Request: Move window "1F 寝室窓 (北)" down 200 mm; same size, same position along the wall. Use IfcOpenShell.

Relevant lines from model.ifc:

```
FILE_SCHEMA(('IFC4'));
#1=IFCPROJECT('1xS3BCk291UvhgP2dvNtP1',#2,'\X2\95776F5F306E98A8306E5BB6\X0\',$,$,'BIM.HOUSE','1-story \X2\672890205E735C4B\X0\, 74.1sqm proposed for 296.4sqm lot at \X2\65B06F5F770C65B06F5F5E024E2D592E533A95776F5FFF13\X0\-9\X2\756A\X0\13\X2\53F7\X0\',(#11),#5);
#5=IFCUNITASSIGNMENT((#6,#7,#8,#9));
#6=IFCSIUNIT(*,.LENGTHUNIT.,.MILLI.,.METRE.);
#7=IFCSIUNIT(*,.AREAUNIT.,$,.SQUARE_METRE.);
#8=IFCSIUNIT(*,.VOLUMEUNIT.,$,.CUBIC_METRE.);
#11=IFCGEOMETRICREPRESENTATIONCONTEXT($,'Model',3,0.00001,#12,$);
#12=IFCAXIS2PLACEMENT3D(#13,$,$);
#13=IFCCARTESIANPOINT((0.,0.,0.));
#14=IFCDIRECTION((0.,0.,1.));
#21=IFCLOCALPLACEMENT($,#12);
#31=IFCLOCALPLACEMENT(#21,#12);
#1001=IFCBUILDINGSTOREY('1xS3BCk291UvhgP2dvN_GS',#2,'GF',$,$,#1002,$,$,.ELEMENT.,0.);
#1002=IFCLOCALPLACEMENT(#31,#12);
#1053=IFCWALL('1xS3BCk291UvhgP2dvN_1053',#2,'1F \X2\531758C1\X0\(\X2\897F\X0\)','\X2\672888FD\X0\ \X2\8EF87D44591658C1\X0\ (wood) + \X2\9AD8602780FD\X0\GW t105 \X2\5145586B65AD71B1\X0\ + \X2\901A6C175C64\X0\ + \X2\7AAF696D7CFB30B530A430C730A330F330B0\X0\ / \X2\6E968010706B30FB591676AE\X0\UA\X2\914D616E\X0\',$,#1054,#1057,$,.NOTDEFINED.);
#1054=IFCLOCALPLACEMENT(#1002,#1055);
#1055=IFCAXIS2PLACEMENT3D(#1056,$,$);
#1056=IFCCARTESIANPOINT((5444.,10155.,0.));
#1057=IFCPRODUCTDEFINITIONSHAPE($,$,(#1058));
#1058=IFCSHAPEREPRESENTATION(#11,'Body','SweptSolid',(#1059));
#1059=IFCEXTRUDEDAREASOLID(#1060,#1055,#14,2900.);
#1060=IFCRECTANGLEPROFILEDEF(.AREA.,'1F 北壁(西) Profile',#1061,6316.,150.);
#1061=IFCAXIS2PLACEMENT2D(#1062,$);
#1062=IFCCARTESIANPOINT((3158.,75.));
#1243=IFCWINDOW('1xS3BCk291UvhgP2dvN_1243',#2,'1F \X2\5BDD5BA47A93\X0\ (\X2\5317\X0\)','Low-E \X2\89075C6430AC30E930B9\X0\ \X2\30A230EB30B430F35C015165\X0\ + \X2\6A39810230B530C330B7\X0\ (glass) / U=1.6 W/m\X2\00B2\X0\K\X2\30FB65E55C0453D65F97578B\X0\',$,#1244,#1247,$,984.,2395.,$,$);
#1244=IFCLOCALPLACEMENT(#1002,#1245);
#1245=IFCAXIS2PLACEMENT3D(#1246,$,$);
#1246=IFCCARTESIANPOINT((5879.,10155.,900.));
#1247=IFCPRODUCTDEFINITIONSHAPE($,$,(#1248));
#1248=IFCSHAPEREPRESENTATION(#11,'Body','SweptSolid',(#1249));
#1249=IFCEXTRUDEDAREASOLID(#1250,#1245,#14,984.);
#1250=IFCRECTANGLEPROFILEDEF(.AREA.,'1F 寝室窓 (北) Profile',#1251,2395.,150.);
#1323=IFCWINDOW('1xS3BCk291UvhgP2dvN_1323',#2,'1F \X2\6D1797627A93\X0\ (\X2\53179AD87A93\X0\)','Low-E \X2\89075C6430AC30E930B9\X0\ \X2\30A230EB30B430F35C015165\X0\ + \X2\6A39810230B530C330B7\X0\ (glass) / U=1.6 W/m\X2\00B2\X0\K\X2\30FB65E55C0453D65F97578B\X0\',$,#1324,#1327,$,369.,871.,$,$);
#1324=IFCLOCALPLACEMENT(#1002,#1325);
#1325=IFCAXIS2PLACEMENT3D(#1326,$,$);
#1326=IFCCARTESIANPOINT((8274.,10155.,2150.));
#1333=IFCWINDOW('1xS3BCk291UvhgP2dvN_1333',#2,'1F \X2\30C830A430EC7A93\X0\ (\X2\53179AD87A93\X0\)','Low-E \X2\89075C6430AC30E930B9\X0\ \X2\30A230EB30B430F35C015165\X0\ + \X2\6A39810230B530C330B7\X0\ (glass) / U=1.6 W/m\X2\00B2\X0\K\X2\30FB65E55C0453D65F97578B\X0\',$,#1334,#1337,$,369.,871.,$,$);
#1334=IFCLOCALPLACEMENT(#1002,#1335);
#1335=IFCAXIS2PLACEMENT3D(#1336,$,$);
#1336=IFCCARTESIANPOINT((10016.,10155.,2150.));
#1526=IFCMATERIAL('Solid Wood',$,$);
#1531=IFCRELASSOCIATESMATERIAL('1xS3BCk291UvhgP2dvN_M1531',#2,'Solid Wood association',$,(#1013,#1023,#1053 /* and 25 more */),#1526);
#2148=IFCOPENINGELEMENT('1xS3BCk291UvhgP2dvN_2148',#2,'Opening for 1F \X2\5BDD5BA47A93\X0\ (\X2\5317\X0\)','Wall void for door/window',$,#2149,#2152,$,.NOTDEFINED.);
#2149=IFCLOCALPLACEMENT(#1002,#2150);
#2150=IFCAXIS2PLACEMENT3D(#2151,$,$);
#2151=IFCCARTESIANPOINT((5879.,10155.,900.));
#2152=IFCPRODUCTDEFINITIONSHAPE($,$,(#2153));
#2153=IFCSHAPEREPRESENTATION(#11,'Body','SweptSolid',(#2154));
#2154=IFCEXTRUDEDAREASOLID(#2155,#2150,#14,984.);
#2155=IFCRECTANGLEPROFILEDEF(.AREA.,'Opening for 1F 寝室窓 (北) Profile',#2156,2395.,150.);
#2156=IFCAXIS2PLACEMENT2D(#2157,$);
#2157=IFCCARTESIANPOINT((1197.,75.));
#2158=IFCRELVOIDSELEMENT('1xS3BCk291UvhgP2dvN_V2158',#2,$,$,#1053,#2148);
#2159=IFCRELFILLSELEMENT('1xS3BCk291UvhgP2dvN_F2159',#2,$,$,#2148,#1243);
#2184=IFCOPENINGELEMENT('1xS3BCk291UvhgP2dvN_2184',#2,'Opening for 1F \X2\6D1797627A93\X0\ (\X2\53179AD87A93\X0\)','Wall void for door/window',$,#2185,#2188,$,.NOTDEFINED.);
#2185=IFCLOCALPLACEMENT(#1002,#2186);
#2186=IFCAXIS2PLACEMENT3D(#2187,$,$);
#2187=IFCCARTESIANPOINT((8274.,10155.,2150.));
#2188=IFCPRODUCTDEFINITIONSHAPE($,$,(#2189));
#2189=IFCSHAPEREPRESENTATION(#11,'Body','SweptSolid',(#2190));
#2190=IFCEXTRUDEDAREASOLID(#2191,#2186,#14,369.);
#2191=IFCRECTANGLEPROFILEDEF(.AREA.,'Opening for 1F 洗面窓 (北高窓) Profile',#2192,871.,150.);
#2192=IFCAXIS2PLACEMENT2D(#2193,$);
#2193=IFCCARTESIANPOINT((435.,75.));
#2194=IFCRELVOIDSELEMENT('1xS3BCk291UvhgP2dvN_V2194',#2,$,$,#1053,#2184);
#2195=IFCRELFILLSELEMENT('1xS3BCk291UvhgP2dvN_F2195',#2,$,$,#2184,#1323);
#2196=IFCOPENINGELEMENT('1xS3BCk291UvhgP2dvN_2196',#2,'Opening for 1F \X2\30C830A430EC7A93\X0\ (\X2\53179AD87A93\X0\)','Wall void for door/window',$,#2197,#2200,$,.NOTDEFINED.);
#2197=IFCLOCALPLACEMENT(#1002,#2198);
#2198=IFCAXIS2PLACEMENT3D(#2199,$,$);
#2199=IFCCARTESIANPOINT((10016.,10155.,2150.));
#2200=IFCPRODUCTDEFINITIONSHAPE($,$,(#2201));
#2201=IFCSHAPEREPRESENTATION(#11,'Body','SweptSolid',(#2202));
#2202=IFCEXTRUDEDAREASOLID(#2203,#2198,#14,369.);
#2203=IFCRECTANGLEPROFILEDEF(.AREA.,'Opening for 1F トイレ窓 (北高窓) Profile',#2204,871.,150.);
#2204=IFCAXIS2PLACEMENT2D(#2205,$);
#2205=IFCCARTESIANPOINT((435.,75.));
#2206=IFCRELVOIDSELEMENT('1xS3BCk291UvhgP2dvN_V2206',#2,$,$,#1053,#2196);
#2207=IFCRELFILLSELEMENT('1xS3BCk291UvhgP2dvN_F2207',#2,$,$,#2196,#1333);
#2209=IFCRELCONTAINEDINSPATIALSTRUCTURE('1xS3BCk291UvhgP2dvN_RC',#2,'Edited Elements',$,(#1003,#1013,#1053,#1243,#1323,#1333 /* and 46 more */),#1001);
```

```python
import numpy as np
import ifcopenshell
import ifcopenshell.api.geometry
import ifcopenshell.util.placement
import ifcopenshell.util.unit

model = ifcopenshell.open("model.ifc")
unit_scale = ifcopenshell.util.unit.calculate_unit_scale(model)

window = model.by_id(1243)
opening = window.FillsVoids[0].RelatingOpeningElement
dz = -200.0

shift = np.array([0.0, 0.0, dz])
# The window is not placed relative to its opening, so move both.
for product in (opening, window):
    matrix = ifcopenshell.util.placement.get_local_placement(product.ObjectPlacement)
    matrix[:3, 3] += shift
    ifcopenshell.api.geometry.edit_object_placement(model, product=product, matrix=matrix, is_si=False)

print(f"moved by {dz * unit_scale:+.3f} m")

model.write("model_edited.ifc")
```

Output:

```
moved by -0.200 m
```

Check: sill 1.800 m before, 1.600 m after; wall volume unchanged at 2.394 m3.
